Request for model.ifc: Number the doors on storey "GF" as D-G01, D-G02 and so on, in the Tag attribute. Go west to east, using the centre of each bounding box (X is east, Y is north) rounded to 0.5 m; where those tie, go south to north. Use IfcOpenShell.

First a look at what the model holds.

```python
import ifcopenshell
import ifcopenshell.util.element
import ifcopenshell.util.placement

model = ifcopenshell.open("model.ifc")
print(model.schema)
storey = next(s for s in model.by_type("IfcBuildingStorey") if s.Name == "GF")
doors = [e for e in ifcopenshell.util.element.get_decomposition(storey) if e.is_a("IfcDoor")]
for e in sorted(doors, key=lambda e: e.id()):
    origin = ifcopenshell.util.placement.get_local_placement(e.ObjectPlacement)[:3, 3]
    print(e.id(), e.Tag, e.Name, origin.round(2) + 0.0, sep=" | ")
```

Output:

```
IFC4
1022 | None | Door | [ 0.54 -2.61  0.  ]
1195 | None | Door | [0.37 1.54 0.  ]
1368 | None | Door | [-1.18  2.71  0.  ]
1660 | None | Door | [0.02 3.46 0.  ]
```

```python
import ifcopenshell
import ifcopenshell.geom
import ifcopenshell.util.element
import ifcopenshell.util.shape

model = ifcopenshell.open("model.ifc")
settings = ifcopenshell.geom.settings()
settings.set("use-world-coords", True)


def centre(element):
    shape = ifcopenshell.geom.create_shape(settings, element)
    return ifcopenshell.util.shape.get_bbox_centroid(shape.geometry)


storey = next(s for s in model.by_type("IfcBuildingStorey") if s.Name == "GF")
doors = [e for e in ifcopenshell.util.element.get_decomposition(storey) if e.is_a("IfcDoor")]

# Insertion points can sit at a corner or the storey origin, so sort by the geometry (in metres).
centres = {e: centre(e) for e in doors}
doors.sort(key=lambda e: (round(centres[e][0] / 0.5), centres[e][1]))

for i, e in enumerate(doors, start=1):
    number = f"D-G{i:02d}"
    e.Tag = number
    print(e.id(), number)

model.write("model_edited.ifc")
```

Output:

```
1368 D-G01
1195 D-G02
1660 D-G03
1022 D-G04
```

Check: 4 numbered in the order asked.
